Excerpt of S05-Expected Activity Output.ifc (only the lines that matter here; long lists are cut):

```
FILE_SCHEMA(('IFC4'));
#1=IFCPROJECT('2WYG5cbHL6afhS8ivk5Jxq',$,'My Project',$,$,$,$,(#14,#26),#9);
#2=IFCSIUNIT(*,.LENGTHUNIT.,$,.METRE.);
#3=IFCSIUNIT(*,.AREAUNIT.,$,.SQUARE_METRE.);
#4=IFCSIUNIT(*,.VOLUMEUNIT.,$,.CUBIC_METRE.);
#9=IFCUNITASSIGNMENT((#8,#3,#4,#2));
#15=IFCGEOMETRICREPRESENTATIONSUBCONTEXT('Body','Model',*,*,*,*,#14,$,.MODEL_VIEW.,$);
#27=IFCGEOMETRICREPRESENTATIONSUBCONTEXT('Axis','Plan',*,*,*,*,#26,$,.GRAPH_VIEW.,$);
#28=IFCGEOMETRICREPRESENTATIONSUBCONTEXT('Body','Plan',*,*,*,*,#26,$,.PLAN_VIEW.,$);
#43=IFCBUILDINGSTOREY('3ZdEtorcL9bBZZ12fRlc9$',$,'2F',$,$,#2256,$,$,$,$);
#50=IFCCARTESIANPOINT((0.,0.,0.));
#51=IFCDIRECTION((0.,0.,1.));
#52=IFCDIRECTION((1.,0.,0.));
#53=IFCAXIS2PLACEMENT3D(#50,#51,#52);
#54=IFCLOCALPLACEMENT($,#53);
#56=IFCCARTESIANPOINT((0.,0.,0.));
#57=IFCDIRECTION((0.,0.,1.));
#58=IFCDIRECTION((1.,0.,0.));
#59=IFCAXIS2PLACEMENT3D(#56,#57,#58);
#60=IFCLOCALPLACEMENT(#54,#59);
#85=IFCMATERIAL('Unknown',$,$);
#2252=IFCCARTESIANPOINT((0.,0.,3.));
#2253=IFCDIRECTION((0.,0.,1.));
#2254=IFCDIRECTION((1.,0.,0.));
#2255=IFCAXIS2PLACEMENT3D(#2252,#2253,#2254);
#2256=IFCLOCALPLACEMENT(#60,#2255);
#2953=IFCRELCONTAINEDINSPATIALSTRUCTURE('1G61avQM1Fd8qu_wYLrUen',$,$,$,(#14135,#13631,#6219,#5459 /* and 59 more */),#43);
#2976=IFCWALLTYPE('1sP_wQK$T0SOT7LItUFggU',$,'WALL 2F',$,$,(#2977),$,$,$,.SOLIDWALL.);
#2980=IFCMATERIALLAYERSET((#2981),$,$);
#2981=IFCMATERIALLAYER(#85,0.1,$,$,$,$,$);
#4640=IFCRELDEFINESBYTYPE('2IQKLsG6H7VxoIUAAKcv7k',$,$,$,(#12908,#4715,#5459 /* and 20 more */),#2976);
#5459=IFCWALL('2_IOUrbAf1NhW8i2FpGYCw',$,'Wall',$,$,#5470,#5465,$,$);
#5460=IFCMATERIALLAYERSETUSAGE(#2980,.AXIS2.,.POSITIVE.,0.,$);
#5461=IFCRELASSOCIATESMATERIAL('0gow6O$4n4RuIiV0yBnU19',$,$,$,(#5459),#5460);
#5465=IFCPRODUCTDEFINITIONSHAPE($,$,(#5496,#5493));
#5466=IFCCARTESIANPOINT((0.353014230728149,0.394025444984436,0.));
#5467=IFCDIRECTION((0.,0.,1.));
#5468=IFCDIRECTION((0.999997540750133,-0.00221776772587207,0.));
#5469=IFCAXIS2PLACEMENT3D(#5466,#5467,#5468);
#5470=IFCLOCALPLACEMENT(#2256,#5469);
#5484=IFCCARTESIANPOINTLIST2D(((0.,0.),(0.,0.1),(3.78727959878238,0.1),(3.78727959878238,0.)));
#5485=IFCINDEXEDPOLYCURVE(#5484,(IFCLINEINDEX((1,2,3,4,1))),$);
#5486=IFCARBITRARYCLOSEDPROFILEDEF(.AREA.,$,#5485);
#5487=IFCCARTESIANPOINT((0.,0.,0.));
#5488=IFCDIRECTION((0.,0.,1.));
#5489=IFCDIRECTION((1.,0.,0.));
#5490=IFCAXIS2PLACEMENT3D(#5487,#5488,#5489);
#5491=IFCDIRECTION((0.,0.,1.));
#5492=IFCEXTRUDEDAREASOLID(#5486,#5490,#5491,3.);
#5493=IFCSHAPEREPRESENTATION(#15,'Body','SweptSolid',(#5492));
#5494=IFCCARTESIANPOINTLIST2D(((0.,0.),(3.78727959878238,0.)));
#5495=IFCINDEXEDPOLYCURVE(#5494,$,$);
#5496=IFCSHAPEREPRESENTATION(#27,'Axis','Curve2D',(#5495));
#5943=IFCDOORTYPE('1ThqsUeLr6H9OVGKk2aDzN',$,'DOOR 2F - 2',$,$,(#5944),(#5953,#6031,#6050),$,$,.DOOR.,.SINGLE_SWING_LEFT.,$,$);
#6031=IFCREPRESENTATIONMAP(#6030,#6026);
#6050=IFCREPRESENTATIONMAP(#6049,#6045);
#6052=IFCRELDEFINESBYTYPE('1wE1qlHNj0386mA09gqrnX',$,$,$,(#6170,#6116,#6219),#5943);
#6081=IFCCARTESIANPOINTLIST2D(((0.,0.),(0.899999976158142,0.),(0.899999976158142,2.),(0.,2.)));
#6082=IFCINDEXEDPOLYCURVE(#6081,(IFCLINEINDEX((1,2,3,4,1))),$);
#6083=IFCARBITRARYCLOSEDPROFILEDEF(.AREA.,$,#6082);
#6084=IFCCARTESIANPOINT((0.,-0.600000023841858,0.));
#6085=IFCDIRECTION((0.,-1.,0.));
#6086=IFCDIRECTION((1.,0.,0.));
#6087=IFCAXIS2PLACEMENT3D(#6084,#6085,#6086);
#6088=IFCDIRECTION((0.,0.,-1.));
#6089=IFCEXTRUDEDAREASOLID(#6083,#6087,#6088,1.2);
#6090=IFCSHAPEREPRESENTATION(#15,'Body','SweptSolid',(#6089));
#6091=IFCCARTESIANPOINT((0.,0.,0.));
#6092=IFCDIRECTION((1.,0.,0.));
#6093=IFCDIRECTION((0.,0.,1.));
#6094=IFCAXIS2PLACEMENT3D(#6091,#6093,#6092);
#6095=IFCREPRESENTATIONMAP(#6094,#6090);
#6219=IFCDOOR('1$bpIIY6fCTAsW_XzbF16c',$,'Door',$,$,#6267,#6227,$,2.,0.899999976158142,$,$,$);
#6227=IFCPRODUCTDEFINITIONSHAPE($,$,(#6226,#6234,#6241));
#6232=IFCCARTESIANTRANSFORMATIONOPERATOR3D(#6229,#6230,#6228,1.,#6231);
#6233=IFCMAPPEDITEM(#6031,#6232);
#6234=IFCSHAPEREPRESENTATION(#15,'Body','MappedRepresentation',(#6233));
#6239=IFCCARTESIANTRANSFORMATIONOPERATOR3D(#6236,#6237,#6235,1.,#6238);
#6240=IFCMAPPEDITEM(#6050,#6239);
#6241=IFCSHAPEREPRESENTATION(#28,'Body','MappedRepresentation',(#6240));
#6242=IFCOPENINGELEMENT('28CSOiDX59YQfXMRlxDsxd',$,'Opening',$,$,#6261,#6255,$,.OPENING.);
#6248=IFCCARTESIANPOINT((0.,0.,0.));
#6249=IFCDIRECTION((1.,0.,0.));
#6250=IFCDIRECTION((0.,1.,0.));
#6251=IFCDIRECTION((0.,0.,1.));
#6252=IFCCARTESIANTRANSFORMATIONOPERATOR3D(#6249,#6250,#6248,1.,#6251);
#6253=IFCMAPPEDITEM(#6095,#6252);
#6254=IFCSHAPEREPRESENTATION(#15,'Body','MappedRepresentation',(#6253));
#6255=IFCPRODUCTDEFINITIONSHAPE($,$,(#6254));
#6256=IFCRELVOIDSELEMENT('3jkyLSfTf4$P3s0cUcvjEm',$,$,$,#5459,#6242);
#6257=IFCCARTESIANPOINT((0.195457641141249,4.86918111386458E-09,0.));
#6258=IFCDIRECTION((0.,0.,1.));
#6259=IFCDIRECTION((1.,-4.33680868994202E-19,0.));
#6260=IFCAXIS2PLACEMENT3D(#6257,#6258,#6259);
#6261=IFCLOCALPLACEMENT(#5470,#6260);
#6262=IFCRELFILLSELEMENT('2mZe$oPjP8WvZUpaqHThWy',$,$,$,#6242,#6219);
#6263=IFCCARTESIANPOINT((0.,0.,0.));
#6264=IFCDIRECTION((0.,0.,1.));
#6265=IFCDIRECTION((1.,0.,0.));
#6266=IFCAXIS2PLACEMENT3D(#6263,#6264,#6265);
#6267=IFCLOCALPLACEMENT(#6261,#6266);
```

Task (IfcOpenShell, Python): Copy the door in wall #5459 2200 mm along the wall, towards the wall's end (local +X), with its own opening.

```python
import ifcopenshell
import ifcopenshell.api.feature
import ifcopenshell.api.geometry
import ifcopenshell.api.root
import ifcopenshell.geom
import ifcopenshell.util.element
import ifcopenshell.util.placement
import ifcopenshell.util.shape
import ifcopenshell.util.unit

model = ifcopenshell.open("S05-Expected Activity Output.ifc")
unit_scale = ifcopenshell.util.unit.calculate_unit_scale(model)
settings = ifcopenshell.geom.settings()


def volume(element):
    """Net volume in cubic metres, openings subtracted."""
    shape = ifcopenshell.geom.create_shape(settings, element)
    return ifcopenshell.util.shape.get_volume(shape.geometry)


door = model.by_guid("1$bpIIY6fCTAsW_XzbF16c")
opening = door.FillsVoids[0].RelatingOpeningElement
wall = opening.VoidsElements[0].RelatingBuildingElement
before = volume(wall)
shift = ifcopenshell.util.placement.get_local_placement(wall.ObjectPlacement)[:3, 0] * 2.2 / unit_scale

# copy_class copies the void relationship, type, container and properties, but no geometry.
new_opening = ifcopenshell.api.root.copy_class(model, product=opening)
new_opening.Representation = ifcopenshell.util.element.copy_deep(
    model, opening.Representation, exclude=["IfcGeometricRepresentationContext", "IfcRepresentationMap"]
)
new_door = ifcopenshell.api.root.copy_class(model, product=door)
new_door.Representation = ifcopenshell.util.element.copy_deep(
    model, door.Representation, exclude=["IfcGeometricRepresentationContext", "IfcRepresentationMap"]
)
ifcopenshell.api.feature.add_filling(model, opening=new_opening, element=new_door)

for old, new in ((opening, new_opening), (door, new_door)):
    matrix = ifcopenshell.util.placement.get_local_placement(old.ObjectPlacement)
    matrix[:3, 3] += shift
    ifcopenshell.api.geometry.edit_object_placement(model, product=new, matrix=matrix, is_si=False)

after = volume(wall)

print(f"wall volume {before:.3f} -> {after:.3f} m3")

model.write("S05-Expected Activity Output-out.ifc")
```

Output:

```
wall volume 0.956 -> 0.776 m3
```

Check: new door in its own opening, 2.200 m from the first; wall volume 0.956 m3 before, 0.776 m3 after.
